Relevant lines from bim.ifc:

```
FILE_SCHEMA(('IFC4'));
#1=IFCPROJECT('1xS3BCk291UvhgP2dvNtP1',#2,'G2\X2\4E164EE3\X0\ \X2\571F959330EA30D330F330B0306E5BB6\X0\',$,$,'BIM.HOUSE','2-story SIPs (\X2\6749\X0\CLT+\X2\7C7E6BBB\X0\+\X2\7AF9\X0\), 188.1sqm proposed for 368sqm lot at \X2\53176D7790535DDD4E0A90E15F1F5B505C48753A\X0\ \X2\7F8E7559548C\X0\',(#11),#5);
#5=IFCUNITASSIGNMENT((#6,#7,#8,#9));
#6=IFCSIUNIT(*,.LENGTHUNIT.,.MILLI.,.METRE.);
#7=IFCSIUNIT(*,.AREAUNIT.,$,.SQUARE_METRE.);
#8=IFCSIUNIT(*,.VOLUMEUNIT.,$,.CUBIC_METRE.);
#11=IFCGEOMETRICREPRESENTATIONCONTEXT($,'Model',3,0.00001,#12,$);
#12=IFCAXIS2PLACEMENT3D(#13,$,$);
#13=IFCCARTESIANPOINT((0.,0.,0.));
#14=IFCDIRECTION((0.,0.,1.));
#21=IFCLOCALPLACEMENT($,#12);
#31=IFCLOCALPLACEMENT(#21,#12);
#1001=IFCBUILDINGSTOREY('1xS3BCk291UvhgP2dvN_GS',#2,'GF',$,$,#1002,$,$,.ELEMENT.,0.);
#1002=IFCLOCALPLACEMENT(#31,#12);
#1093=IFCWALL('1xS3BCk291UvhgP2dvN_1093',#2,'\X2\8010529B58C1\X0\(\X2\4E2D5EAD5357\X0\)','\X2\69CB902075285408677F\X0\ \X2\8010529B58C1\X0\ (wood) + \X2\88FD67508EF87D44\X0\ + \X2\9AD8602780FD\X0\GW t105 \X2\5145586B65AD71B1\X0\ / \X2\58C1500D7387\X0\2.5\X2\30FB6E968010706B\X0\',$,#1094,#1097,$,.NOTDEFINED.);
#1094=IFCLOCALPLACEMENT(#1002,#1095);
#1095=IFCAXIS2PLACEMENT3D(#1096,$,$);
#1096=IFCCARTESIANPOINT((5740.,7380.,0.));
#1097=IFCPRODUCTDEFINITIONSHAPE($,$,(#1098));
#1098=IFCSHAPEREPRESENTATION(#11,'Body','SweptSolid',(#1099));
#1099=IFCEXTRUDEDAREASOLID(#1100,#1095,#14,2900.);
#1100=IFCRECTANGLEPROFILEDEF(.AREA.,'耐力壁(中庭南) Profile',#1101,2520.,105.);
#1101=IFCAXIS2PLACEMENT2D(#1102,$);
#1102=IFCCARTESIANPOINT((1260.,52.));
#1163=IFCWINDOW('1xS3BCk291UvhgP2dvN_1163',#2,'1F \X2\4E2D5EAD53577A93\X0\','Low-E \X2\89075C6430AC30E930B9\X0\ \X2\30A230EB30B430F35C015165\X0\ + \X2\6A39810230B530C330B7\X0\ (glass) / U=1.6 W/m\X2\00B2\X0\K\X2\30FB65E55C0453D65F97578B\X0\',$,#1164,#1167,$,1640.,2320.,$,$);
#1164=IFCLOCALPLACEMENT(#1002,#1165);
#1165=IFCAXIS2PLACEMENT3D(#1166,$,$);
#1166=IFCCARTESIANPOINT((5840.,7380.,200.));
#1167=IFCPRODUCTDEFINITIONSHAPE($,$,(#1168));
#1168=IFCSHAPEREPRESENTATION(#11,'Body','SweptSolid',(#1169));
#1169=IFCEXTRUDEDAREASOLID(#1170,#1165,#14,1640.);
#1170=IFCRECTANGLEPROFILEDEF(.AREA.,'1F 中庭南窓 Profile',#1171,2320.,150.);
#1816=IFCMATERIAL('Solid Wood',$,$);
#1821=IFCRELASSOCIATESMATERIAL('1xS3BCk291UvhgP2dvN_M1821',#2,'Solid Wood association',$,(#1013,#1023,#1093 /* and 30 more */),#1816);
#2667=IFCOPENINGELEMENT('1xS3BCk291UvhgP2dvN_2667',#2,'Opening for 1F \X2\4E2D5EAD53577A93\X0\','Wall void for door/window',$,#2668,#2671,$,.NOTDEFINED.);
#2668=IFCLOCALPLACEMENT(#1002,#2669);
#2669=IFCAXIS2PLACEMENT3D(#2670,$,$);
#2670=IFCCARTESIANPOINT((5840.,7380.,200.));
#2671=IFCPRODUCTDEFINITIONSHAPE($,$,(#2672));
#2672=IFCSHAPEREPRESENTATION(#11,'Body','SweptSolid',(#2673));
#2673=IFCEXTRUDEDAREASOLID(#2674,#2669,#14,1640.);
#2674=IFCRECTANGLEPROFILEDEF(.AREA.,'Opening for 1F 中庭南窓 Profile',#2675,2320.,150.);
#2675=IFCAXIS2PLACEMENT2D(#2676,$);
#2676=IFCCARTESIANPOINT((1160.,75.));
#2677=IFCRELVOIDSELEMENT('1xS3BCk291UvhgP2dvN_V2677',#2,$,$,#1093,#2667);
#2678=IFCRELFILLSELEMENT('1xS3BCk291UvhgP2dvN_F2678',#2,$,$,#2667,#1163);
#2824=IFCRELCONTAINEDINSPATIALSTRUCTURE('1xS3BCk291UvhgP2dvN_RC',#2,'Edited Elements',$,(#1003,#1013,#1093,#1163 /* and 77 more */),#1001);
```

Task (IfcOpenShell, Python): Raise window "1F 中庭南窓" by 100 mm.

```python
import numpy as np
import ifcopenshell
import ifcopenshell.api.geometry
import ifcopenshell.util.placement
import ifcopenshell.util.unit

model = ifcopenshell.open("bim.ifc")
unit_scale = ifcopenshell.util.unit.calculate_unit_scale(model)

window = model.by_guid("1xS3BCk291UvhgP2dvN_1163")
opening = window.FillsVoids[0].RelatingOpeningElement
dz = 100.0

shift = np.array([0.0, 0.0, dz])
# The window is not placed relative to its opening, so move both.
for product in (opening, window):
    matrix = ifcopenshell.util.placement.get_local_placement(product.ObjectPlacement)
    matrix[:3, 3] += shift
    ifcopenshell.api.geometry.edit_object_placement(model, product=product, matrix=matrix, is_si=False)

print(f"moved by {dz * unit_scale:+.3f} m")

model.write("bim_updated.ifc")
```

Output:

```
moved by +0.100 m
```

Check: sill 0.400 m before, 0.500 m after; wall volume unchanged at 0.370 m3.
